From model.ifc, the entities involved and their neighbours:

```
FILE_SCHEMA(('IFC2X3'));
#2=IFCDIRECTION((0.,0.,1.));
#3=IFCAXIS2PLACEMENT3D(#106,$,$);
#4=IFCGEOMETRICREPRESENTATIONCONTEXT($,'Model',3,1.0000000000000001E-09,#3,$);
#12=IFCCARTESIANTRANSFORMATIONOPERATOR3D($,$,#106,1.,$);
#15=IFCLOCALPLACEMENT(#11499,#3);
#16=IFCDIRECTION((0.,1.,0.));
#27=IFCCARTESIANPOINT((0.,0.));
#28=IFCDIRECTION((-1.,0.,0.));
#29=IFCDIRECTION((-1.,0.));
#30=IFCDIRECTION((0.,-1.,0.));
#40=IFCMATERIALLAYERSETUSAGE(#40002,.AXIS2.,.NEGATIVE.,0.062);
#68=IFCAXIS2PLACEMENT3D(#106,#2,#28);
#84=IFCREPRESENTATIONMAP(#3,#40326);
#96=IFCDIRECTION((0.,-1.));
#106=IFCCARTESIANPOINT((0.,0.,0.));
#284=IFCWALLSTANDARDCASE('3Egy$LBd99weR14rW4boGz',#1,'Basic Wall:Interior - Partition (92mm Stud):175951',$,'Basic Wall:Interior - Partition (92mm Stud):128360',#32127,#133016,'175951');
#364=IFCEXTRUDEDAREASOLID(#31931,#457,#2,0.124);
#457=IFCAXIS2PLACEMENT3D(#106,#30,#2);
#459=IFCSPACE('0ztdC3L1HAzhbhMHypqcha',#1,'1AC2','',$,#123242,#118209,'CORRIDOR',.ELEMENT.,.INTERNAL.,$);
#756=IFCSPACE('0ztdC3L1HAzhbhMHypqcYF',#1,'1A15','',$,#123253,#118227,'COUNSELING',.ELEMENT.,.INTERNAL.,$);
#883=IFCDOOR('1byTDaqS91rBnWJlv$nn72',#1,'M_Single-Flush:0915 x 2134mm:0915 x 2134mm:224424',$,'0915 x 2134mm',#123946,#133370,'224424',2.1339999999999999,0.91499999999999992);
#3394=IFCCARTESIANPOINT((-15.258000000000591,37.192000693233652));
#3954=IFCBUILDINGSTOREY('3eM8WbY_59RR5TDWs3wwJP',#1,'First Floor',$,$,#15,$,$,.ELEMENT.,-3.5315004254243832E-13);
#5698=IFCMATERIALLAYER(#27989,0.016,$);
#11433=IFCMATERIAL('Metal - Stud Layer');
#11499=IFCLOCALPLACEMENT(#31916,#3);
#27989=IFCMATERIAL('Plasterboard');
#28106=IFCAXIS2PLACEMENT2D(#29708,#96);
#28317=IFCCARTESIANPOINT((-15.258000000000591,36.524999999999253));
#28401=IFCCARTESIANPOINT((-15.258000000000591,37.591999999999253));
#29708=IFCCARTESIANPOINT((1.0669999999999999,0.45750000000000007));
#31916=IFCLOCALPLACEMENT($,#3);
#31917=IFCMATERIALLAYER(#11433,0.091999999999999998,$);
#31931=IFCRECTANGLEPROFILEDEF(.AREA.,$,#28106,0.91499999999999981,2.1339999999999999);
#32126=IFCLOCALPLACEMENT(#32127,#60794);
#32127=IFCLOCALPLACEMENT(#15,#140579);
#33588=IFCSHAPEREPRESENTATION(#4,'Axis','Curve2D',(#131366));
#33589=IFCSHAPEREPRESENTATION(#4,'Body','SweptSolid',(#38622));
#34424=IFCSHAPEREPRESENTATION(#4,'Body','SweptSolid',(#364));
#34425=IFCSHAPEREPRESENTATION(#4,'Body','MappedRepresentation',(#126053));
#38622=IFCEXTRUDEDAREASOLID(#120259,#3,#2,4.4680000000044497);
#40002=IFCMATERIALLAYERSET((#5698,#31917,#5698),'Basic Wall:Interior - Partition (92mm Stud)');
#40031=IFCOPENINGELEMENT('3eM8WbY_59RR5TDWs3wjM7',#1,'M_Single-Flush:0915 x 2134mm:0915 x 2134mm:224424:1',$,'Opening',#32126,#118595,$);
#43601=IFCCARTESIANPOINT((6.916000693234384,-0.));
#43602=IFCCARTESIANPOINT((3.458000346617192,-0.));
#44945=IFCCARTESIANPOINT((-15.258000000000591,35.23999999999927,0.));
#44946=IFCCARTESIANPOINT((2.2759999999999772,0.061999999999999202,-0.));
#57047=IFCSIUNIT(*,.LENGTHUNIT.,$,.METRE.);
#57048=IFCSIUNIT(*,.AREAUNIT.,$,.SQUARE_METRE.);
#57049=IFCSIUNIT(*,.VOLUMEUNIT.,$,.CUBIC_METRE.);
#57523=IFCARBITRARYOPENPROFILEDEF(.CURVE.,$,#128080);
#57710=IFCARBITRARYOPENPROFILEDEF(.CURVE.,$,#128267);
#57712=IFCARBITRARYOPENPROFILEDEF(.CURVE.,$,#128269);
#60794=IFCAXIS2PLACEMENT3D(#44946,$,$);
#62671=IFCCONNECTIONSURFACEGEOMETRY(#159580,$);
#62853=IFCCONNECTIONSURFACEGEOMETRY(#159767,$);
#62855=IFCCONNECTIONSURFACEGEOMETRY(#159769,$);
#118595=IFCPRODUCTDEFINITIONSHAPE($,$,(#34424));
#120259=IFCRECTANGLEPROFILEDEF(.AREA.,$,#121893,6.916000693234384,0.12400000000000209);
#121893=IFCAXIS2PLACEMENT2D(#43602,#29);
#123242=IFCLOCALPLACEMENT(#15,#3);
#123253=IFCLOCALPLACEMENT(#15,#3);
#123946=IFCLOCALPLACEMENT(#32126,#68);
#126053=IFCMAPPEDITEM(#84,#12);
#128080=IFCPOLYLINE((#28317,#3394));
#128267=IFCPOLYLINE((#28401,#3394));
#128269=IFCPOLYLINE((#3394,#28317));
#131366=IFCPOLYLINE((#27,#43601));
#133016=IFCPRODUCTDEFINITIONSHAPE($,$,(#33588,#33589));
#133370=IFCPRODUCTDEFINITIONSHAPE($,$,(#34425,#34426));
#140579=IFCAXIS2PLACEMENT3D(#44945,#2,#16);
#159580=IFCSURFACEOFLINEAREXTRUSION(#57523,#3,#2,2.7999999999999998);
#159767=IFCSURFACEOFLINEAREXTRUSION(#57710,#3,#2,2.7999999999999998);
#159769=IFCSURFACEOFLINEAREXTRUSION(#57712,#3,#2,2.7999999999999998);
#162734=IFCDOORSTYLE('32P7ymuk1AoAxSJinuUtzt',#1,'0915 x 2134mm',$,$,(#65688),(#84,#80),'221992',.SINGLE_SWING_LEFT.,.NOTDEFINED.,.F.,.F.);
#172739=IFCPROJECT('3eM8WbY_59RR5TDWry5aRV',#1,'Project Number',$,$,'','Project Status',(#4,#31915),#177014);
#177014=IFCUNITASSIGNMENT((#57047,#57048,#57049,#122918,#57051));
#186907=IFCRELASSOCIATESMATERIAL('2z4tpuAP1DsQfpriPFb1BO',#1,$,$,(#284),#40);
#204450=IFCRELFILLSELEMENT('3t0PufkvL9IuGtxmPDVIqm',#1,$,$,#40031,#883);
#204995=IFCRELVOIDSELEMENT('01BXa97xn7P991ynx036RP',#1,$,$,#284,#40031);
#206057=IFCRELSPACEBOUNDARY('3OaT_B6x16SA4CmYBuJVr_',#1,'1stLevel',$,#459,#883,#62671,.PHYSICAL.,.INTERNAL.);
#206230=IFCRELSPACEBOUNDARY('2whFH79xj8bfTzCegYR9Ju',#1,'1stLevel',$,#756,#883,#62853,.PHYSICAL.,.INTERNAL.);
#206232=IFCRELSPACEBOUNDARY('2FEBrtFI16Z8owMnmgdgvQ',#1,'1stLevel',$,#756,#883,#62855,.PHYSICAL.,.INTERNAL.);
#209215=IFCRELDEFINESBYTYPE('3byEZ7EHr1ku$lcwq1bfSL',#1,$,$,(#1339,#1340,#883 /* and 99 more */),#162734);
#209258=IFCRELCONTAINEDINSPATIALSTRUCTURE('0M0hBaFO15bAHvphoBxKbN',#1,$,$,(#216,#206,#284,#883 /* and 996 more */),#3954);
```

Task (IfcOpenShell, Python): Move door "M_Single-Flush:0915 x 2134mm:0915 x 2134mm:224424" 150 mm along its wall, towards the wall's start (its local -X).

```python
import numpy as np
import ifcopenshell
import ifcopenshell.api.geometry
import ifcopenshell.util.placement
import ifcopenshell.util.unit

model = ifcopenshell.open("model.ifc")
unit_scale = ifcopenshell.util.unit.calculate_unit_scale(model)

door = model.by_guid("1byTDaqS91rBnWJlv$nn72")
opening = door.FillsVoids[0].RelatingOpeningElement
wall = opening.VoidsElements[0].RelatingBuildingElement

wall_matrix = ifcopenshell.util.placement.get_local_placement(wall.ObjectPlacement)
shift = wall_matrix[:3, 0] * -0.15 / unit_scale
before = ifcopenshell.util.placement.get_local_placement(door.ObjectPlacement)[:3, 3].copy()

# The door is placed relative to its opening, so it follows when the opening moves.
matrix = ifcopenshell.util.placement.get_local_placement(opening.ObjectPlacement)
matrix[:3, 3] += shift
ifcopenshell.api.geometry.edit_object_placement(
    model, product=opening, matrix=matrix, is_si=False, should_transform_children=True
)

# Space boundary surfaces are stored in each space's coordinates; move them too.
for rel in door.ProvidesBoundaries:
    if not rel.ConnectionGeometry:
        continue
    surface = rel.ConnectionGeometry.SurfaceOnRelatingElement
    space_matrix = ifcopenshell.util.placement.get_local_placement(rel.RelatingSpace.ObjectPlacement)
    point = np.array(surface.Position.Location.Coordinates) + space_matrix[:3, :3].T @ shift
    surface.Position = model.createIfcAxis2Placement3D(
        model.createIfcCartesianPoint(point.tolist()), surface.Position.Axis, surface.Position.RefDirection
    )

after = ifcopenshell.util.placement.get_local_placement(door.ObjectPlacement)[:3, 3]
print("door moved by", (after - before).round(3) + 0.0)

model.write("model_edited.ifc")
```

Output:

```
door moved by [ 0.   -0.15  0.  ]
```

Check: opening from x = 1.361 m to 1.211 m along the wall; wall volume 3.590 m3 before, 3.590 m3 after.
